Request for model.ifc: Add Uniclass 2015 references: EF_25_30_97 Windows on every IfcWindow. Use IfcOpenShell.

First a look at what the model holds.

```python
import ifcopenshell

model = ifcopenshell.open("model.ifc")
print(model.schema)
print("classifications:", [c.Name for c in model.by_type("IfcClassification")])
for ifc_class in ("IfcDoor", "IfcRoof", "IfcStair", "IfcWall", "IfcWindow"):
    print(ifc_class, len(model.by_type(ifc_class)))
```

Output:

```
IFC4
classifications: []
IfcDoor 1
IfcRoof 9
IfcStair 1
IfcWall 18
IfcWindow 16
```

```python
import ifcopenshell
import ifcopenshell.api.classification

model = ifcopenshell.open("model.ifc")

system = ifcopenshell.api.classification.add_classification(model, classification="Uniclass 2015")

codes = {
    "IfcWindow": ("EF_25_30_97", "Windows"),
}
for ifc_class, (code, name) in codes.items():
    products = model.by_type(ifc_class)
    ifcopenshell.api.classification.add_reference(
        model, products=products, classification=system, identification=code, name=name
    )
    print(code, len(products))

model.write("model-out.ifc")
```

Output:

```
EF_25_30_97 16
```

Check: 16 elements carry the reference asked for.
